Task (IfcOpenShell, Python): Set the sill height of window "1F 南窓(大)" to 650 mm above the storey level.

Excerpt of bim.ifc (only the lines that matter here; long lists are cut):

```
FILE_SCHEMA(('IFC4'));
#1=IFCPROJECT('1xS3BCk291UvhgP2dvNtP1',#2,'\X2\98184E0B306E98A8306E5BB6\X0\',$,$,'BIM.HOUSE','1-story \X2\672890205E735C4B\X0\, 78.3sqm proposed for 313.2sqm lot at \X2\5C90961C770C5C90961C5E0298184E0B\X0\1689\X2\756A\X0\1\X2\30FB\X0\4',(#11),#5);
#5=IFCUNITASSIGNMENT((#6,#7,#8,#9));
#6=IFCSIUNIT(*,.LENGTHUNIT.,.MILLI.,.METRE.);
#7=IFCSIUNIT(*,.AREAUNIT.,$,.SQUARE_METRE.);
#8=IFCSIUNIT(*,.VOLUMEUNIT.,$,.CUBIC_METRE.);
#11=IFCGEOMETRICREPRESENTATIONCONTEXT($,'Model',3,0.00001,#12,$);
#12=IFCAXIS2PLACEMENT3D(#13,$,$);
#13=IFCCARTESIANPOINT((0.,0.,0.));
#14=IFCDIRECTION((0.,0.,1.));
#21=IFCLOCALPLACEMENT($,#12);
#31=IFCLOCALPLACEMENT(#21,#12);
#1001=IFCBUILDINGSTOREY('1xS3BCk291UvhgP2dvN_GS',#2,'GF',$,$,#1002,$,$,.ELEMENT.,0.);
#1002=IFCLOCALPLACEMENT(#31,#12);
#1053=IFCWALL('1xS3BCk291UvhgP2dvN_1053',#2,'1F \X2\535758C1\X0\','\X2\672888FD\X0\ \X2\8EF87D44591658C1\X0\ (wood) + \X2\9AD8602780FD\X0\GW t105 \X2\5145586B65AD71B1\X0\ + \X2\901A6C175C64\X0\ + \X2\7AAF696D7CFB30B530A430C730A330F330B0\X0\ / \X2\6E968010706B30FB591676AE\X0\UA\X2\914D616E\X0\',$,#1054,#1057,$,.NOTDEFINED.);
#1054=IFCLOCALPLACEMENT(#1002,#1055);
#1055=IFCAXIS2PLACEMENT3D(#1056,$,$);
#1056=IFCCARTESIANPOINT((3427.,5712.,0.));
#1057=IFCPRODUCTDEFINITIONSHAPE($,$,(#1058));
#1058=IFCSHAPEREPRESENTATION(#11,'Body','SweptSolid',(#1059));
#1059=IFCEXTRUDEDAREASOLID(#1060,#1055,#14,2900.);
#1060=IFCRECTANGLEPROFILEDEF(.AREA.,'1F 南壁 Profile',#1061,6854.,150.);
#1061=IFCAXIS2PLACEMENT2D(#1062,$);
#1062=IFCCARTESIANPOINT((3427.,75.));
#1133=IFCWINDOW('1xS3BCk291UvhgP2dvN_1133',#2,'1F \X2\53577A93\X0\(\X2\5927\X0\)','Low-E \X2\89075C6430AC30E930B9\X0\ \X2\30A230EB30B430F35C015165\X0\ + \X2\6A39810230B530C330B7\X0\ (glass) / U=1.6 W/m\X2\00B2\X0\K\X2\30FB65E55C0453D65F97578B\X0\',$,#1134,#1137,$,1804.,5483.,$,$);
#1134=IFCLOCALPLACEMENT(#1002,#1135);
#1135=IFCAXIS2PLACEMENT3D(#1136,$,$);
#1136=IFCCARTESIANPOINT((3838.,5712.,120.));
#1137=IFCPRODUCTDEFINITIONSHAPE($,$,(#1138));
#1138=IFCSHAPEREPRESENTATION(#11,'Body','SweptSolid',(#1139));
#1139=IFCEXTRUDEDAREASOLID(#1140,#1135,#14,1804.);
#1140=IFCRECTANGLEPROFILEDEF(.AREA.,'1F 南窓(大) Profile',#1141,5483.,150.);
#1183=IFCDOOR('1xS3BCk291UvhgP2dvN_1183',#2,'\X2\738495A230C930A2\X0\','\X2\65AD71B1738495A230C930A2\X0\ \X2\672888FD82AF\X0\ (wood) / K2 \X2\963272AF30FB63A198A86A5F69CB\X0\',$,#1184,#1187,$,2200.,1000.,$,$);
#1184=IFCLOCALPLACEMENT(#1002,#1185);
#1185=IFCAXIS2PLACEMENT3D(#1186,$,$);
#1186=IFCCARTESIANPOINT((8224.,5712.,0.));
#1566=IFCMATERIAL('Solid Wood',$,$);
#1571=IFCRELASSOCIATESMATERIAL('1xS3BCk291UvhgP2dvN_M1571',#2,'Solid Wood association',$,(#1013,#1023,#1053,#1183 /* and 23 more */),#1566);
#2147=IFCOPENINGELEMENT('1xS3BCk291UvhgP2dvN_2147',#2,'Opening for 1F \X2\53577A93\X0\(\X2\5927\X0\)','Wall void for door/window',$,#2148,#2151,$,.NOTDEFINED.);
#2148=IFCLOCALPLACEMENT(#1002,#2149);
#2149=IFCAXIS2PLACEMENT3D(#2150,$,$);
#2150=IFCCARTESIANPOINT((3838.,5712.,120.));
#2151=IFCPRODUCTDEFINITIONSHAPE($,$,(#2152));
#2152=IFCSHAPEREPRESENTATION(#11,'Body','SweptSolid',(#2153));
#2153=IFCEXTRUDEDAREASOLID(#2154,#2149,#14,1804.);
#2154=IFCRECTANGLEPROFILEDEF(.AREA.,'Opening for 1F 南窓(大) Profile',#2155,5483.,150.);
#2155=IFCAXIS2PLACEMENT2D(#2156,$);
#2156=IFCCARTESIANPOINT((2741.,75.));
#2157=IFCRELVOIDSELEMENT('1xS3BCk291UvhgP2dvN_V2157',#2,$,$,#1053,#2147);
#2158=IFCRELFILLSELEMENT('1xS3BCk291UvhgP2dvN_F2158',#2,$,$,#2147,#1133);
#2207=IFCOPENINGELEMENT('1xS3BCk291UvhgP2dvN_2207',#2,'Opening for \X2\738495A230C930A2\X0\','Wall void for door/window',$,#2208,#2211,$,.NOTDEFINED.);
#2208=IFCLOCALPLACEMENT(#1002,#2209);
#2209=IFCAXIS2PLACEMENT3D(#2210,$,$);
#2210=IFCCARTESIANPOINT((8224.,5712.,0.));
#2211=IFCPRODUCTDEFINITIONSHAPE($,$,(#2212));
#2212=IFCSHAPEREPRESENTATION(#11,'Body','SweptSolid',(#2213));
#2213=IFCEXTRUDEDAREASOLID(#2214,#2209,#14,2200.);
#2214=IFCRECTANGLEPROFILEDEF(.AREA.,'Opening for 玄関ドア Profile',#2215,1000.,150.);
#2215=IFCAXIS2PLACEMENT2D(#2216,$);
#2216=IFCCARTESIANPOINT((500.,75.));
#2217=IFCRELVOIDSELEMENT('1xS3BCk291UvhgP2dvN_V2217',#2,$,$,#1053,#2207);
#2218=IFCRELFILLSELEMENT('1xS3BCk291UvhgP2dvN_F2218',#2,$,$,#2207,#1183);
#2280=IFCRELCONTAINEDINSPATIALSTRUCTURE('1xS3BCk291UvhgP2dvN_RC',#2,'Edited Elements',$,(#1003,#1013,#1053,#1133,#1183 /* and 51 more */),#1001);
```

```python
import numpy as np
import ifcopenshell
import ifcopenshell.api.geometry
import ifcopenshell.geom
import ifcopenshell.util.element
import ifcopenshell.util.placement
import ifcopenshell.util.shape
import ifcopenshell.util.unit

model = ifcopenshell.open("bim.ifc")
unit_scale = ifcopenshell.util.unit.calculate_unit_scale(model)

window = model.by_id(1133)
opening = window.FillsVoids[0].RelatingOpeningElement
storey = ifcopenshell.util.element.get_container(window, ifc_class="IfcBuildingStorey")
level = ifcopenshell.util.placement.get_local_placement(storey.ObjectPlacement)[2, 3]

# The opening's origin need not be at the sill, so measure its lowest point.
shape = ifcopenshell.geom.create_shape(ifcopenshell.geom.settings(), opening)
bottom = ifcopenshell.util.shape.get_shape_bottom_elevation(shape, shape.geometry) / unit_scale
dz = level + 650.0 - bottom

shift = np.array([0.0, 0.0, dz])
# The window is not placed relative to its opening, so move both.
for product in (opening, window):
    matrix = ifcopenshell.util.placement.get_local_placement(product.ObjectPlacement)
    matrix[:3, 3] += shift
    ifcopenshell.api.geometry.edit_object_placement(model, product=product, matrix=matrix, is_si=False)

print(f"moved by {dz * unit_scale:+.3f} m")

model.write("bim_v2.ifc")
```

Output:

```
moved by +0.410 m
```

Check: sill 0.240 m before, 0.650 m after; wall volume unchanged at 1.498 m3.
